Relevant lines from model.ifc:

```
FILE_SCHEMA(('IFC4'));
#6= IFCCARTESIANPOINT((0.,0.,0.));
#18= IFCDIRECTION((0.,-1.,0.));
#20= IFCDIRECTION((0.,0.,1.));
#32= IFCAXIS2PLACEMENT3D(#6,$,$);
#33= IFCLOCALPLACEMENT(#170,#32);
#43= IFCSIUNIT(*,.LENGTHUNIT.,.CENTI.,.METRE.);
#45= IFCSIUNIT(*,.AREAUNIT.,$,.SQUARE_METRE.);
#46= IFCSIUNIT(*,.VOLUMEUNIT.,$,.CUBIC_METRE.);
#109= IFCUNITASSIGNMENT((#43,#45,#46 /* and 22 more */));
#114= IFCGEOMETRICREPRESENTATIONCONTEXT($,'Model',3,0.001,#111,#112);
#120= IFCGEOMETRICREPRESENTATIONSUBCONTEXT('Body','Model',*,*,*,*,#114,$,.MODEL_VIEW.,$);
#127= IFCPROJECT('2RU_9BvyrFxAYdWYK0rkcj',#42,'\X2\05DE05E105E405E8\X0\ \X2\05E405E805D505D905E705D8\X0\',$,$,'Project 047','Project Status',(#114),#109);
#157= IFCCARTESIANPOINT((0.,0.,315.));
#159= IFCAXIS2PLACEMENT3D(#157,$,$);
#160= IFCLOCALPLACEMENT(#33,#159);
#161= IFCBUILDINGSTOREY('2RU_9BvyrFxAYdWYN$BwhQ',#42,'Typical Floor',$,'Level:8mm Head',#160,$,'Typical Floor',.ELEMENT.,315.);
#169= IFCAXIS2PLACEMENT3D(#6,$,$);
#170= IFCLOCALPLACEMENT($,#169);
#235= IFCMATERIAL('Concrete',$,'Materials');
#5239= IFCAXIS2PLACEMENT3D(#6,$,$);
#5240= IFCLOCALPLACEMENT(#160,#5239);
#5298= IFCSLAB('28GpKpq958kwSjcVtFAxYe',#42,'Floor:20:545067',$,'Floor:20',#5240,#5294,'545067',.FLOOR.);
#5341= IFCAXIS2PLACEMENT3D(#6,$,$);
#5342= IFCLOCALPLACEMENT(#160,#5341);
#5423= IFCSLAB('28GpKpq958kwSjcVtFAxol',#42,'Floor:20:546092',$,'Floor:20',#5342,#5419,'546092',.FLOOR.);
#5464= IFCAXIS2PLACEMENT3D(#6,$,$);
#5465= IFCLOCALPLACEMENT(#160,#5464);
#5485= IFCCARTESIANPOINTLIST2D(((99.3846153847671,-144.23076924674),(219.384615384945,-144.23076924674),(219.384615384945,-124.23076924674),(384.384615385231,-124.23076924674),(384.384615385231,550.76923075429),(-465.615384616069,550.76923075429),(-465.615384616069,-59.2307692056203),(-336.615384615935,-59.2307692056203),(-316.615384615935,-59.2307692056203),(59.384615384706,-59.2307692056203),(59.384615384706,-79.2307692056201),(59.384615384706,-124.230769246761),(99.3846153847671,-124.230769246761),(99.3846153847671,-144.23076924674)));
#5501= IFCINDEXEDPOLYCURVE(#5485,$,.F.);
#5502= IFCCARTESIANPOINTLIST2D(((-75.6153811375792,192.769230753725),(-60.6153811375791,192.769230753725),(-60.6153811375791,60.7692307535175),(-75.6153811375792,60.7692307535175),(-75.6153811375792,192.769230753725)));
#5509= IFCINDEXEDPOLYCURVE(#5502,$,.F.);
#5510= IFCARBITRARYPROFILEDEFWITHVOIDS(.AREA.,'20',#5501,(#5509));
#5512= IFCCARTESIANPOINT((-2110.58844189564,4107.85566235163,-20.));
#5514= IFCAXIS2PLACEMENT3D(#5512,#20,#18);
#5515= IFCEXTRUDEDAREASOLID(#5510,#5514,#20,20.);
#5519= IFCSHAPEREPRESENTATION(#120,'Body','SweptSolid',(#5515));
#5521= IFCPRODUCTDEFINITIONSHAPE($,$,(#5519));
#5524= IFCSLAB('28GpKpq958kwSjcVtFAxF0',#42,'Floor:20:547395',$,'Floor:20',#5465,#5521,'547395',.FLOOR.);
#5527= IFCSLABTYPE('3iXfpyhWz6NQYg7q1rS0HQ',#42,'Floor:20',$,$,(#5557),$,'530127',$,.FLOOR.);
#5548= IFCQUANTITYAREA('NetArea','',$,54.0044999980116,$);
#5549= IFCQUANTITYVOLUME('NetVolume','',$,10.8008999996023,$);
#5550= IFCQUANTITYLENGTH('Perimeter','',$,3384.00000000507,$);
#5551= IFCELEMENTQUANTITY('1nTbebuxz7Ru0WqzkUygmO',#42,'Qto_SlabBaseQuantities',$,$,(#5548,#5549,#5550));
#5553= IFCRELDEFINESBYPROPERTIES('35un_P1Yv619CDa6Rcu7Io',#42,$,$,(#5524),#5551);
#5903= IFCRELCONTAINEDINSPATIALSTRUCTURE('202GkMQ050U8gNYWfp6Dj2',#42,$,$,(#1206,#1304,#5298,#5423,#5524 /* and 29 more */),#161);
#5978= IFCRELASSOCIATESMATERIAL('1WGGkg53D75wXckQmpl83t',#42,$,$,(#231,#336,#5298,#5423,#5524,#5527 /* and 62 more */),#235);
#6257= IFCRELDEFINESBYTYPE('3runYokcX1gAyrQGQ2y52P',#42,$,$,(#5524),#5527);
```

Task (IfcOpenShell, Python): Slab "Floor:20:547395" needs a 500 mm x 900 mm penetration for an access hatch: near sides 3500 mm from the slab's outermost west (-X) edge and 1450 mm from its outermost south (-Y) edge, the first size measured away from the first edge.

```python
import numpy as np
import ifcopenshell
import ifcopenshell.api.feature
import ifcopenshell.api.geometry
import ifcopenshell.api.pset
import ifcopenshell.api.root
import ifcopenshell.geom
import ifcopenshell.util.element
import ifcopenshell.util.placement
import ifcopenshell.util.representation
import ifcopenshell.util.shape
import ifcopenshell.util.unit

model = ifcopenshell.open("model.ifc")
unit_scale = ifcopenshell.util.unit.calculate_unit_scale(model)
area_scale = ifcopenshell.util.unit.calculate_unit_scale(model, "AREAUNIT")
volume_scale = ifcopenshell.util.unit.calculate_unit_scale(model, "VOLUMEUNIT")
settings = ifcopenshell.geom.settings()


def volume(element):
    """Net volume in cubic metres, openings subtracted."""
    shape = ifcopenshell.geom.create_shape(settings, element)
    return ifcopenshell.util.shape.get_volume(shape.geometry)


slab = model.by_guid("28GpKpq958kwSjcVtFAxF0")
before = volume(slab)

# Extent in the slab's own axes, in metres. The edges named are its -X and -Y sides.
slab_shape = ifcopenshell.geom.create_shape(settings, slab)
vertices = ifcopenshell.util.shape.get_vertices(slab_shape.geometry)
x_min, y_min, bottom = vertices.min(axis=0)
top = vertices[:, 2].max()

opening = ifcopenshell.api.root.create_entity(model, ifc_class="IfcOpeningElement", name="Access hatch opening", predefined_type="OPENING")
context = ifcopenshell.util.representation.get_context(model, "Model", "Body", "MODEL_VIEW")
width, depth = 0.5, 0.9
outline = [(0.0, 0.0), (width, 0.0), (width, depth), (0.0, depth), (0.0, 0.0)]
# Overshoot both faces by 50 mm so the cut is clean.
shape = ifcopenshell.api.geometry.add_slab_representation(
    model, context=context, depth=top - bottom + 0.1, polyline=outline
)
ifcopenshell.api.geometry.assign_representation(model, product=opening, representation=shape)

matrix = ifcopenshell.util.placement.get_local_placement(slab.ObjectPlacement)
matrix[:, 3] = matrix @ np.append(np.array([x_min + 3.5, y_min + 1.45, bottom - 0.05]) / unit_scale, 1.0)
ifcopenshell.api.geometry.edit_object_placement(model, product=opening, matrix=matrix, is_si=False)
ifcopenshell.api.feature.add_feature(model, feature=opening, element=slab)

after = volume(slab)

# Update the slab's stored quantities.
qto = model.by_id(ifcopenshell.util.element.get_pset(slab, "Qto_SlabBaseQuantities", should_inherit=False)["id"])
ifcopenshell.api.pset.edit_qto(model, qto=qto, properties={
    "NetArea": after / (top - bottom) / area_scale,
    "NetVolume": after / volume_scale,
})

print(f"slab volume {before:.3f} -> {after:.3f} m3")

model.write("model-out.ifc")
```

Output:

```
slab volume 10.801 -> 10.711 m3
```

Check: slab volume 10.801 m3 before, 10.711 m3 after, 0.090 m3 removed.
